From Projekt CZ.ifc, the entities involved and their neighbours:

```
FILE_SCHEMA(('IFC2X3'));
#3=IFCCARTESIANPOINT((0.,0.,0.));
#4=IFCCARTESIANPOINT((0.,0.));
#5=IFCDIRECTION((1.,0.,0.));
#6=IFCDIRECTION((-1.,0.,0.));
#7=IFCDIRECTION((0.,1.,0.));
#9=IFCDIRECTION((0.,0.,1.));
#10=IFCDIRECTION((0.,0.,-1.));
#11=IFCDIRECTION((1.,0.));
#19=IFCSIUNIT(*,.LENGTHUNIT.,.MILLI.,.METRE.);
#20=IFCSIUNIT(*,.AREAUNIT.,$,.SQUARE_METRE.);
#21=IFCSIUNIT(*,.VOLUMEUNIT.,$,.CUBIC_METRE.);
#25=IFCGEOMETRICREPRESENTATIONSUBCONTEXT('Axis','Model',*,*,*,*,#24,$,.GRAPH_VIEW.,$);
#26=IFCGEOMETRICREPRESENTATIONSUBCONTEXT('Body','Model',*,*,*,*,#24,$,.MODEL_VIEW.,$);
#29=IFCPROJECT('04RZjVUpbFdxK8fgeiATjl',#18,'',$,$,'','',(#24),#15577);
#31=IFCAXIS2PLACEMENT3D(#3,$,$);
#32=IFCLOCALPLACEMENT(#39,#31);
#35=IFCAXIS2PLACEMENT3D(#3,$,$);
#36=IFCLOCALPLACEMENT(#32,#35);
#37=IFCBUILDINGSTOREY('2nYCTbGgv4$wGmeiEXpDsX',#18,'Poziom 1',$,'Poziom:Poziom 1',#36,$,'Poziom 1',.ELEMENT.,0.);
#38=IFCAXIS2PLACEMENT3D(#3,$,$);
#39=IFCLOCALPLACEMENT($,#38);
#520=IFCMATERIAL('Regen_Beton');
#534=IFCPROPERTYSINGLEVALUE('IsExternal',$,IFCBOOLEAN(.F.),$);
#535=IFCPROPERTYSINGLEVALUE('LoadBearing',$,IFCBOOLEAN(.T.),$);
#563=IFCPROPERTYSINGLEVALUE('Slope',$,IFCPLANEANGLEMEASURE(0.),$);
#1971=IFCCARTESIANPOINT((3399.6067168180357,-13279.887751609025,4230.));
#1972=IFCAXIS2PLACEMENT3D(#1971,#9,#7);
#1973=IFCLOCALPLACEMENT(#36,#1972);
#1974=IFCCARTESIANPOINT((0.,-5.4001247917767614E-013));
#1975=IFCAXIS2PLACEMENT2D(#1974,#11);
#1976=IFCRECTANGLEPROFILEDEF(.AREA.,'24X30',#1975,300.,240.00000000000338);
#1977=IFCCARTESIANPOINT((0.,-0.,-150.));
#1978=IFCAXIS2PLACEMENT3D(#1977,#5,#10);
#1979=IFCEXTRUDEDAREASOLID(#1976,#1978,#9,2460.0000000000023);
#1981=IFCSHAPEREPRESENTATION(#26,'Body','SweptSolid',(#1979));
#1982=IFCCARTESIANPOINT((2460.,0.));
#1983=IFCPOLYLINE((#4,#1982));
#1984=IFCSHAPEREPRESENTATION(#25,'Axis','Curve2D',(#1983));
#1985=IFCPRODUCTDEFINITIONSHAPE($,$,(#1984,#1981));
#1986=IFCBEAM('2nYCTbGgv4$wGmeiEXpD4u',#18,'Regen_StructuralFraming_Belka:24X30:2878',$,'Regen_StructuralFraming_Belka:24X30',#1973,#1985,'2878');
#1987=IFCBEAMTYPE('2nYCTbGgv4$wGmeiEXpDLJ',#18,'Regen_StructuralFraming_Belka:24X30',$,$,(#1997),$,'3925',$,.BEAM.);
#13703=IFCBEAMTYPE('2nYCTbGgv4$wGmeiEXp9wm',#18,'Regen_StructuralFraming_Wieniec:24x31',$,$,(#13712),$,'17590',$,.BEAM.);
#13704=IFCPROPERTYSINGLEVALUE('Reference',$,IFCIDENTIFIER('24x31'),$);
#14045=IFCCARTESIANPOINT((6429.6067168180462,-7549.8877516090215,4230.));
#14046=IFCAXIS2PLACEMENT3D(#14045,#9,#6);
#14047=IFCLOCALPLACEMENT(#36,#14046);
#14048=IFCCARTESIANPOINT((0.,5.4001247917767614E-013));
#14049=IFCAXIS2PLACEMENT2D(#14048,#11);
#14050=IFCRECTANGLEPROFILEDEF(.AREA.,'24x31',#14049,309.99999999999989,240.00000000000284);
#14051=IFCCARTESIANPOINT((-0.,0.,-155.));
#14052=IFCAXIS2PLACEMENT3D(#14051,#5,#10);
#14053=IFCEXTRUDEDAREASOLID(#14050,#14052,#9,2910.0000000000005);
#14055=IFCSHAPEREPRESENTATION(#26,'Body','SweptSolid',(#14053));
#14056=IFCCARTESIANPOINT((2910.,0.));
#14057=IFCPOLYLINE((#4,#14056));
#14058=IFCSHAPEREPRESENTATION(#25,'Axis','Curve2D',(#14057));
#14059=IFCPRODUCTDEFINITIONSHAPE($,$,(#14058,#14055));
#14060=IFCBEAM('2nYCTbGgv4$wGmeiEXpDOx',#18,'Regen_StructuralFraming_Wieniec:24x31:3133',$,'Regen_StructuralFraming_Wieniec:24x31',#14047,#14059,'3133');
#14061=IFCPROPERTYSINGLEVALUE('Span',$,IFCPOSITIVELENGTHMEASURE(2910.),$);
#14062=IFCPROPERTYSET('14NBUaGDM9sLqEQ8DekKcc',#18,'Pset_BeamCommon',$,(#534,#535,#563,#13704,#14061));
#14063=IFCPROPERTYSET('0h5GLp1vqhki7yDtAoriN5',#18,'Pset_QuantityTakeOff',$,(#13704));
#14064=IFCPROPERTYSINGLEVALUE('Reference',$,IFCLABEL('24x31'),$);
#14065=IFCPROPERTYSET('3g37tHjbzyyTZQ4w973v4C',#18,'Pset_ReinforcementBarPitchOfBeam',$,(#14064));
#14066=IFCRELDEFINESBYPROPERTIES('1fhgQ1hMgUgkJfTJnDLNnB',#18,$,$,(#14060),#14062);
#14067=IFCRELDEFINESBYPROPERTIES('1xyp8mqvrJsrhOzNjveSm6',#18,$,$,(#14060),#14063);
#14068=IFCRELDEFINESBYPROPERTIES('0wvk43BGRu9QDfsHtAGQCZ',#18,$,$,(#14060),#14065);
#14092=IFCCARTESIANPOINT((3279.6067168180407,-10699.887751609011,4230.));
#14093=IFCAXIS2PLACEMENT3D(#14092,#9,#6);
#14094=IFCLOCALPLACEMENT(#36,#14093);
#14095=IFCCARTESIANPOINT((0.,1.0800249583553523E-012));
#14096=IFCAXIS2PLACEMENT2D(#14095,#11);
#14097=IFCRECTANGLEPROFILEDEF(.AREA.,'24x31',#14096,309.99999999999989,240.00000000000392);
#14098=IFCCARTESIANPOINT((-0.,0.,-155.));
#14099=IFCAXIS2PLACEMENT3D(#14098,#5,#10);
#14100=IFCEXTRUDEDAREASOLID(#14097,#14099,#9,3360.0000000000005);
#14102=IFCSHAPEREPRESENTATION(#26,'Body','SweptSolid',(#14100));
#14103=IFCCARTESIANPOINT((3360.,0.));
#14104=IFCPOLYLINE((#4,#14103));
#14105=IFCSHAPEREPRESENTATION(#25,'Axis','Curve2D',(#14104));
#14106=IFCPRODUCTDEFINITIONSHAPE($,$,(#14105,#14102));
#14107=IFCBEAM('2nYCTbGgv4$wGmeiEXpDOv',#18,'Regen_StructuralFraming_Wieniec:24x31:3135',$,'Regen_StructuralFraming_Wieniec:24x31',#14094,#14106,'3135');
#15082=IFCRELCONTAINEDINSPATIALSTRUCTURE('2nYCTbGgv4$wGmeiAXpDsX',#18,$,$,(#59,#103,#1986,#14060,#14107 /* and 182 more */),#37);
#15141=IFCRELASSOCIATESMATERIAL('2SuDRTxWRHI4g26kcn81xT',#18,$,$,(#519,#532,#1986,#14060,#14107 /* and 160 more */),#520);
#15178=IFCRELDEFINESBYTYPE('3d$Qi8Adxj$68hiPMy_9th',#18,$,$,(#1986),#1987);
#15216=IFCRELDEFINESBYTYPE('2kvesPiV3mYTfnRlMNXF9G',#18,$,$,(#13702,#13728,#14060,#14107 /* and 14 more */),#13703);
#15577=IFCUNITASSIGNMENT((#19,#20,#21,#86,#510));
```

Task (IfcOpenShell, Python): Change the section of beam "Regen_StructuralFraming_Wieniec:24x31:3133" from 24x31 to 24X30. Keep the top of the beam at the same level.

```python
import ifcopenshell
import ifcopenshell.api.pset
import ifcopenshell.api.type
import ifcopenshell.util.element
import ifcopenshell.util.representation

model = ifcopenshell.open("Projekt CZ.ifc")

member = model.by_guid("2nYCTbGgv4$wGmeiEXpDOx")
source = next(p for p in model.by_type("IfcRectangleProfileDef") if p.ProfileName == "24X30")

body = ifcopenshell.util.representation.get_representation(member, "Model", "Body")
solid = body.Items[0]
old_profile = solid.SweptArea

# Copy the section's sizes but keep this member's own profile position.
profile = ifcopenshell.util.element.copy(model, source)
# Profiles are centred, so shift by half the change in depth to hold the top.
shift = (old_profile.XDim - profile.XDim) / 2
x, y = old_profile.Position.Location.Coordinates
up = (-1.0, 0.0)  # upwards, in the solid's own plane
location = model.createIfcCartesianPoint((x + up[0] * shift, y + up[1] * shift))
profile.Position = model.createIfcAxis2Placement2D(location, old_profile.Position.RefDirection)
solid.SweptArea = profile
if not model.get_total_inverses(old_profile):
    ifcopenshell.util.element.remove_deep2(model, old_profile)

new_type = model.by_guid("2nYCTbGgv4$wGmeiEXpDLJ")
ifcopenshell.api.type.assign_type(
    model, related_objects=[member], relating_type=new_type, should_map_representations=False
)
member.Name = member.Name.replace("24x31", "24X30")
member.ObjectType = "Regen_StructuralFraming_Wieniec:24X30"
pset = model.by_id(ifcopenshell.util.element.get_pset(member, "Pset_BeamCommon", should_inherit=False)["id"])
ifcopenshell.api.pset.edit_pset(model, pset=pset, properties={"Reference": "24X30"})
pset = model.by_id(ifcopenshell.util.element.get_pset(member, "Pset_QuantityTakeOff", should_inherit=False)["id"])
ifcopenshell.api.pset.edit_pset(model, pset=pset, properties={"Reference": "24X30"})
pset = model.by_id(ifcopenshell.util.element.get_pset(member, "Pset_ReinforcementBarPitchOfBeam", should_inherit=False)["id"])
ifcopenshell.api.pset.edit_pset(model, pset=pset, properties={"Reference": "24X30"})

print(solid.SweptArea)

model.write("Projekt CZ_updated.ifc")
```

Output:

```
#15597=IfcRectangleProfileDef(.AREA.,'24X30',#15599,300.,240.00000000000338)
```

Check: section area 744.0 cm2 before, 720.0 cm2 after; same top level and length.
